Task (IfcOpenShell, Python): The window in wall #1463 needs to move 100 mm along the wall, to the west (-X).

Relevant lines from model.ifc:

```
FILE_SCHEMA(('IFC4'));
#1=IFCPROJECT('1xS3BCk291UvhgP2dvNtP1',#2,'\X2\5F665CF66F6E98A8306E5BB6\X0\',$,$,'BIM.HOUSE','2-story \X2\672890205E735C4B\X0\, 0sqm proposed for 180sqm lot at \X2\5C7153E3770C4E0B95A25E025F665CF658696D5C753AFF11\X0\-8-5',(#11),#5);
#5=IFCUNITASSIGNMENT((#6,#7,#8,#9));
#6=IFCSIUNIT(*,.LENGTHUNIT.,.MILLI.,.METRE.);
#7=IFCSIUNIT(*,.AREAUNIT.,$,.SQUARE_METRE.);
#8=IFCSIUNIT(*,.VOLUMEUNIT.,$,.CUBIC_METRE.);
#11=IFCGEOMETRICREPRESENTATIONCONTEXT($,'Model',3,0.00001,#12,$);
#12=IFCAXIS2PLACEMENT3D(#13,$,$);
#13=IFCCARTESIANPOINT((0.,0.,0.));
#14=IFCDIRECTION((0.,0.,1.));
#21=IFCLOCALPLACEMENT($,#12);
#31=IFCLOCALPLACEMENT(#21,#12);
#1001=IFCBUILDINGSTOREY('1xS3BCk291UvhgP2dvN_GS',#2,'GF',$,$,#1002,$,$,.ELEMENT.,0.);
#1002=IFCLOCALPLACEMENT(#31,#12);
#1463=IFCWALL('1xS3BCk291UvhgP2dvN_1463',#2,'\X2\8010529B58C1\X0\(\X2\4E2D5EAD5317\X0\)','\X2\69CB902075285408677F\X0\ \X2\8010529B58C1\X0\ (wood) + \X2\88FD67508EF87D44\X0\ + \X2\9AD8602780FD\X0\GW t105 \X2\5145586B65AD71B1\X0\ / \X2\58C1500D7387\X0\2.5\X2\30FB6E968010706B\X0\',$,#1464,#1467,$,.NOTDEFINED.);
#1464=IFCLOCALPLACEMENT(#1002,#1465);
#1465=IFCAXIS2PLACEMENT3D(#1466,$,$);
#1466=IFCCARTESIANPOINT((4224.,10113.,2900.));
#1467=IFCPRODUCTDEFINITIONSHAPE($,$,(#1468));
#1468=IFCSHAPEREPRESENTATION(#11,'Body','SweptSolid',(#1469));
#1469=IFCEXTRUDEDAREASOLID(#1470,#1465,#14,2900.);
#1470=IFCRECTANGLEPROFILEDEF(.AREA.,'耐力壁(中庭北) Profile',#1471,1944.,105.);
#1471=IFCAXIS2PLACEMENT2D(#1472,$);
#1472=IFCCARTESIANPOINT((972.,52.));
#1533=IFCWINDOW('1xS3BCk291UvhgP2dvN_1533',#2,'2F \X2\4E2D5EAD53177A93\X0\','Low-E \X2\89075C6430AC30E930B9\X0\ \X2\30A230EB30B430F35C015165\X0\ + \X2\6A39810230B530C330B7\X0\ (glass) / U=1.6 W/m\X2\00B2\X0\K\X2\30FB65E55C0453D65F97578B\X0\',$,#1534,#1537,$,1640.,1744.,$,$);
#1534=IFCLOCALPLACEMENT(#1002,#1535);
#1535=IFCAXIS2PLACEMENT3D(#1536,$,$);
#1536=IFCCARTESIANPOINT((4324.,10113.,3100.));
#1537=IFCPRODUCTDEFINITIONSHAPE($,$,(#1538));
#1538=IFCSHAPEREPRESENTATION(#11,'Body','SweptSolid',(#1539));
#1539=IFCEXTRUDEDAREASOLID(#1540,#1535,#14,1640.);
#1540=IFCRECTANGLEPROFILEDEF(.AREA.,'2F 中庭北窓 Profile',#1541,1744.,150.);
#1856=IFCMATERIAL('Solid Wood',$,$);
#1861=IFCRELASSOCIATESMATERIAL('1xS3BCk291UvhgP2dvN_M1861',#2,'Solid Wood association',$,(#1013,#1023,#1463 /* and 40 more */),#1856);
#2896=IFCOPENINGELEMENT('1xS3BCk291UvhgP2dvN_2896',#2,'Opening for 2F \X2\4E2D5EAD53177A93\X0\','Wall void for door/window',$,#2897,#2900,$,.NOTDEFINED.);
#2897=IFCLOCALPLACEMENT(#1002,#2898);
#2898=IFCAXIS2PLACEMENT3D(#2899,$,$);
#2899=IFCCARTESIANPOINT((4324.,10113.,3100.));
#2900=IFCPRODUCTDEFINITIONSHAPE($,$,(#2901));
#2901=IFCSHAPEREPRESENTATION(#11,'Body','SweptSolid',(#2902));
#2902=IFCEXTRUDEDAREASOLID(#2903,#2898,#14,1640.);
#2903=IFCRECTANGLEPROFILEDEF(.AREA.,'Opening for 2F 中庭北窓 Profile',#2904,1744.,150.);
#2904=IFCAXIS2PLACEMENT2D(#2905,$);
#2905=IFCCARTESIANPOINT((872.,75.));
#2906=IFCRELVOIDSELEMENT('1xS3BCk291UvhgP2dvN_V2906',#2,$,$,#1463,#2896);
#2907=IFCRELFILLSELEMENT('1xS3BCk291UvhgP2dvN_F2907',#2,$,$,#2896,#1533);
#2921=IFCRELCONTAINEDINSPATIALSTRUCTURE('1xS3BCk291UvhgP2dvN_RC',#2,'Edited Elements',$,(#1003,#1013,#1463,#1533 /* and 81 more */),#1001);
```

```python
import ifcopenshell
import ifcopenshell.api.geometry
import ifcopenshell.util.placement

model = ifcopenshell.open("model.ifc")

window = model.by_guid("1xS3BCk291UvhgP2dvN_1533")
opening = window.FillsVoids[0].RelatingOpeningElement
wall = opening.VoidsElements[0].RelatingBuildingElement

wall_matrix = ifcopenshell.util.placement.get_local_placement(wall.ObjectPlacement)
shift = wall_matrix[:3, 0] * -100.0
before = ifcopenshell.util.placement.get_local_placement(window.ObjectPlacement)[:3, 3].copy()

# The window is not placed relative to its opening, so move both.
for product in (opening, window):
    matrix = ifcopenshell.util.placement.get_local_placement(product.ObjectPlacement)
    matrix[:3, 3] += shift
    ifcopenshell.api.geometry.edit_object_placement(model, product=product, matrix=matrix, is_si=False)

after = ifcopenshell.util.placement.get_local_placement(window.ObjectPlacement)[:3, 3]
print("window moved by", (after - before).round(3) + 0.0)

model.write("model_edited.ifc")
```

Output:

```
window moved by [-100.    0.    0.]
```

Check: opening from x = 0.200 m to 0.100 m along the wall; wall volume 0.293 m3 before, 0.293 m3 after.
